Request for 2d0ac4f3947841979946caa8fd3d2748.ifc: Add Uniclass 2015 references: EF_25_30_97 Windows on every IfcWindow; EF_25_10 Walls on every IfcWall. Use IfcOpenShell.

First a look at what the model holds.

```python
import ifcopenshell

model = ifcopenshell.open("2d0ac4f3947841979946caa8fd3d2748.ifc")
print(model.schema)
print("classifications:", [c.Name for c in model.by_type("IfcClassification")])
for ifc_class in ("IfcDoor", "IfcRoof", "IfcStair", "IfcWall", "IfcWindow"):
    print(ifc_class, len(model.by_type(ifc_class)))
```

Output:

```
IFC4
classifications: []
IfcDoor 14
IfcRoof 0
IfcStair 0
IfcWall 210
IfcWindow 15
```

```python
import ifcopenshell
import ifcopenshell.api.classification

model = ifcopenshell.open("2d0ac4f3947841979946caa8fd3d2748.ifc")

system = ifcopenshell.api.classification.add_classification(model, classification="Uniclass 2015")

codes = {
    "IfcWindow": ("EF_25_30_97", "Windows"),
    "IfcWall": ("EF_25_10", "Walls"),
}
for ifc_class, (code, name) in codes.items():
    products = model.by_type(ifc_class)
    ifcopenshell.api.classification.add_reference(
        model, products=products, classification=system, identification=code, name=name
    )
    print(code, len(products))

model.write("2d0ac4f3947841979946caa8fd3d2748_edited.ifc")
```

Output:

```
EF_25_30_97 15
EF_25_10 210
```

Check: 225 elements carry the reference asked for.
